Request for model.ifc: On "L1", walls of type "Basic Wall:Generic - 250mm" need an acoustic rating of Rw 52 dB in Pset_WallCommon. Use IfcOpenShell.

First a look at what the model holds.

```python
import ifcopenshell
import ifcopenshell.util.element

model = ifcopenshell.open("model.ifc")
print(model.schema)
storey = next(s for s in model.by_type("IfcBuildingStorey") if s.Name == "L1")
walls = [e for e in ifcopenshell.util.element.get_decomposition(storey) if e.is_a("IfcWall")]
seen = {}
for e in walls:
    element_type = ifcopenshell.util.element.get_type(e)
    key = (element_type.Name if element_type != e and element_type else None, ifcopenshell.util.element.get_pset(e, "Pset_WallCommon", "AcousticRating"))
    seen[key] = seen.get(key, 0) + 1
for (name, value), count in sorted(seen.items(), key=str):
    print(count, "x", name, "|", value)
```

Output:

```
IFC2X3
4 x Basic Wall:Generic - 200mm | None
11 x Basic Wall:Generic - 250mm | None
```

```python
import ifcopenshell
import ifcopenshell.api.pset
import ifcopenshell.util.element

model = ifcopenshell.open("model.ifc")

storey = next(s for s in model.by_type("IfcBuildingStorey") if s.Name == "L1")
walls = [e for e in ifcopenshell.util.element.get_decomposition(storey) if e.is_a("IfcWall")]

count = 0
for e in walls:
    element_type = ifcopenshell.util.element.get_type(e)
    if element_type in (None, e) or element_type.Name != "Basic Wall:Generic - 250mm":
        continue
    # add_pset returns the element's existing set when there is one.
    pset = ifcopenshell.api.pset.add_pset(model, product=e, name="Pset_WallCommon")
    ifcopenshell.api.pset.edit_pset(model, pset=pset, properties={"AcousticRating": "Rw 52 dB"})
    count += 1

print(count, "walls updated")

model.write("model-out.ifc")
```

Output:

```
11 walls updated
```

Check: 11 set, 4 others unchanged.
